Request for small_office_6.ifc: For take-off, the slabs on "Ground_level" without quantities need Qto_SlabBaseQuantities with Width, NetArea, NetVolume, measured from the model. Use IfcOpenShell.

First a look at what the model holds.

```python
import ifcopenshell
import ifcopenshell.util.element
import ifcopenshell.util.unit

model = ifcopenshell.open("small_office_6.ifc")
print(model.schema)
for unit_type in ("LENGTHUNIT", "AREAUNIT", "VOLUMEUNIT"):
    print(unit_type, ifcopenshell.util.unit.calculate_unit_scale(model, unit_type))
storey = next(s for s in model.by_type("IfcBuildingStorey") if s.Name == "Ground_level")
slabs = [e for e in ifcopenshell.util.element.get_decomposition(storey) if e.is_a("IfcSlab")]
for e in sorted(slabs, key=lambda e: e.id()):
    print(e.id(), e.is_a(), e.Name, list(ifcopenshell.util.element.get_psets(e, qtos_only=True)), sep=" | ")
```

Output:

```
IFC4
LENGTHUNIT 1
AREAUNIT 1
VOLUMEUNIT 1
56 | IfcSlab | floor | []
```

```python
import ifcopenshell
import ifcopenshell.api.pset
import ifcopenshell.geom
import ifcopenshell.util.element
import ifcopenshell.util.shape
import ifcopenshell.util.unit

model = ifcopenshell.open("small_office_6.ifc")
unit_scale = ifcopenshell.util.unit.calculate_unit_scale(model)
area_scale = ifcopenshell.util.unit.calculate_unit_scale(model, "AREAUNIT")
volume_scale = ifcopenshell.util.unit.calculate_unit_scale(model, "VOLUMEUNIT")
settings = ifcopenshell.geom.settings()

storey = next(s for s in model.by_type("IfcBuildingStorey") if s.Name == "Ground_level")
slabs = [e for e in ifcopenshell.util.element.get_decomposition(storey) if e.is_a("IfcSlab")]

for e in sorted(slabs, key=lambda e: e.id()):
    if ifcopenshell.util.element.get_psets(e, qtos_only=True, should_inherit=False):
        continue
    # Geometry comes back in metres, in the element's own axes.
    shape = ifcopenshell.geom.create_shape(settings, e)
    values = {
        "Width": ifcopenshell.util.shape.get_z(shape.geometry) / unit_scale,
        "NetArea": ifcopenshell.util.shape.get_footprint_area(shape.geometry) / area_scale,
        "NetVolume": ifcopenshell.util.shape.get_volume(shape.geometry) / volume_scale,
    }
    qto = ifcopenshell.api.pset.add_qto(model, product=e, name="Qto_SlabBaseQuantities")
    ifcopenshell.api.pset.edit_qto(model, qto=qto, properties=values)
    print(e.id(), {k: round(v, 3) for k, v in values.items()})

model.write("small_office_6-out.ifc")
```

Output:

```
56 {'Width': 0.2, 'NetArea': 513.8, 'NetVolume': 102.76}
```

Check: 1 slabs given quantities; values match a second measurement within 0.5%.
